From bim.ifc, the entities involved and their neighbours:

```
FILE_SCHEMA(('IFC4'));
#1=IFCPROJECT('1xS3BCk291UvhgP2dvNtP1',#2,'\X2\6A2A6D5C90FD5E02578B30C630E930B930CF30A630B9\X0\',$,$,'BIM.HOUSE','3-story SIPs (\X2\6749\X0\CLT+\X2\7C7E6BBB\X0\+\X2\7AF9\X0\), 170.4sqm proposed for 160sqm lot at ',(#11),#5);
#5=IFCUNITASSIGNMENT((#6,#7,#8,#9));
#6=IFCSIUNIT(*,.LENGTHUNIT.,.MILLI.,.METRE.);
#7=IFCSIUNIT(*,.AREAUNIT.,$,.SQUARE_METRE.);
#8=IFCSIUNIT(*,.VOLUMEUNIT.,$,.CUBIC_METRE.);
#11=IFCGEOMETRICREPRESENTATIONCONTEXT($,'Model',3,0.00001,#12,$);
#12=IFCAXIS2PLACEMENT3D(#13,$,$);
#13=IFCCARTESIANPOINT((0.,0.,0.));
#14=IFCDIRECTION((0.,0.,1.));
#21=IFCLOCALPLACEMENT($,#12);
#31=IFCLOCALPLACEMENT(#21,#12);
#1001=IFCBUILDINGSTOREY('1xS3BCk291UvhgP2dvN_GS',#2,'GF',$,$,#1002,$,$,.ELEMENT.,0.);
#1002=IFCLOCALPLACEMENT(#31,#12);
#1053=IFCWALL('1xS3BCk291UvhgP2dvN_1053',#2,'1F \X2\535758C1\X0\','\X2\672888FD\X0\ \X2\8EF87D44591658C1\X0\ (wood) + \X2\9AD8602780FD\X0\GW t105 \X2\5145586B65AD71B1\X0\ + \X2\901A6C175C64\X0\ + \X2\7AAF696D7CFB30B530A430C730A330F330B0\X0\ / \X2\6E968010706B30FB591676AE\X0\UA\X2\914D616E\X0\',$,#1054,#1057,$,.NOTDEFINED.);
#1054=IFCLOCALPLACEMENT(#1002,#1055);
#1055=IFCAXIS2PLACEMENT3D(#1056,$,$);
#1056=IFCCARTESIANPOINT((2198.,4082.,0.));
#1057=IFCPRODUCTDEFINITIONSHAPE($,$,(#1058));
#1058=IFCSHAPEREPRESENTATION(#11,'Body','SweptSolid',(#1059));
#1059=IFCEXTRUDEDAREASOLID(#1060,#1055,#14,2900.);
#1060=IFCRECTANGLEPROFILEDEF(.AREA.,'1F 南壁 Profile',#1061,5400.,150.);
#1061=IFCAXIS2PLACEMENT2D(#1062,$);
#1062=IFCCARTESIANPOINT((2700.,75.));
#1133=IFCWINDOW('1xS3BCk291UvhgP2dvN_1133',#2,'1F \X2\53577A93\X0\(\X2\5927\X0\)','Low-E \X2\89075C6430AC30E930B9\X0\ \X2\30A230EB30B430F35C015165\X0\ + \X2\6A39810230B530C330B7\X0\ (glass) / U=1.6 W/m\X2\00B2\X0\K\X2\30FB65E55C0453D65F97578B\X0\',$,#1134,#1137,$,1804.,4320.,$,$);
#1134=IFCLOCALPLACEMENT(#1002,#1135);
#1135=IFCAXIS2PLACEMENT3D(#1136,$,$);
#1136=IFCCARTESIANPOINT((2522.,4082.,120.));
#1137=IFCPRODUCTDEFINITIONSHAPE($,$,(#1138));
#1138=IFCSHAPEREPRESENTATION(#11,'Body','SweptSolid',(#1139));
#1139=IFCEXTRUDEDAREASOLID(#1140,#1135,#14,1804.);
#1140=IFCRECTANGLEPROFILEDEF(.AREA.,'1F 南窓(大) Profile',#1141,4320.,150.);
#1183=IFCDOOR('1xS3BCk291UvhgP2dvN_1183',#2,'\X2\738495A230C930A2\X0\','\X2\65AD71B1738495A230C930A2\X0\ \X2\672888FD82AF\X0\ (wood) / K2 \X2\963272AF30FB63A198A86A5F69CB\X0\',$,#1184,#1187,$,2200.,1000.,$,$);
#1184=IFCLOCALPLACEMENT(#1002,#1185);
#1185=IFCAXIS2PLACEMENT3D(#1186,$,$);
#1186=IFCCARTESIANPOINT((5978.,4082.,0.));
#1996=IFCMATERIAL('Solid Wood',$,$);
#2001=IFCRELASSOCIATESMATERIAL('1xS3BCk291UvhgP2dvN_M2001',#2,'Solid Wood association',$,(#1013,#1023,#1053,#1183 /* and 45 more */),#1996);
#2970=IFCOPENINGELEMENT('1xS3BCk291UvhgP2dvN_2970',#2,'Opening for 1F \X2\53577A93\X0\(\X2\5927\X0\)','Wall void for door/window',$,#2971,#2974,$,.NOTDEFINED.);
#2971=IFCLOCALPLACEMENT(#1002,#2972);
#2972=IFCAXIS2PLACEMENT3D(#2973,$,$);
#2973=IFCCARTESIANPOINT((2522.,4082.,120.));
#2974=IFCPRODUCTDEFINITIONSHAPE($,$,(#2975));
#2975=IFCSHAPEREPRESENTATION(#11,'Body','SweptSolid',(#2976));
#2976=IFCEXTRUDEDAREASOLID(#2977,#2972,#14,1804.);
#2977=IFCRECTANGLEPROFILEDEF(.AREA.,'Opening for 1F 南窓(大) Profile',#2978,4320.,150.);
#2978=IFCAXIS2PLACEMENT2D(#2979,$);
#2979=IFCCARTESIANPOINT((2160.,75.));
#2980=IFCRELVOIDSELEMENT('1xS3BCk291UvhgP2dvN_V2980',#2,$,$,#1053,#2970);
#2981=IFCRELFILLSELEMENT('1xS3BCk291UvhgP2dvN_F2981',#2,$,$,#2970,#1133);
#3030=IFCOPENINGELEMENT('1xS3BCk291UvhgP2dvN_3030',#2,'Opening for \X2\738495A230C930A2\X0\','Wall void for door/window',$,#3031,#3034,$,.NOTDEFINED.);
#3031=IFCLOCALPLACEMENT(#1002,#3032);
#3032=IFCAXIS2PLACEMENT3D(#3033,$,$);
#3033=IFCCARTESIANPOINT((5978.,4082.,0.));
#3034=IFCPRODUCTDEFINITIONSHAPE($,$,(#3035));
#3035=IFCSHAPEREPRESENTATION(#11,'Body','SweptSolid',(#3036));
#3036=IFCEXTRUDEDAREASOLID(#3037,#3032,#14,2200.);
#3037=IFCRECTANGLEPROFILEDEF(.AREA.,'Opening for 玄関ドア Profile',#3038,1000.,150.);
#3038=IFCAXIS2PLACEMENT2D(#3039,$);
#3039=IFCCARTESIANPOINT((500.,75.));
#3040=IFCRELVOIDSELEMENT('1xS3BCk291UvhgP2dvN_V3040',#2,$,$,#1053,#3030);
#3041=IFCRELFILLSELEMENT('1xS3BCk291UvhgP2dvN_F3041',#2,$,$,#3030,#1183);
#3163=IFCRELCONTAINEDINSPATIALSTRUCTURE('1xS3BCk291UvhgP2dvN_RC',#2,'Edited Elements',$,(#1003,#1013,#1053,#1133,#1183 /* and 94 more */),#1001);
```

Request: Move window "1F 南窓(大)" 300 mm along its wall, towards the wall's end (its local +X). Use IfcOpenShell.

```python
import ifcopenshell
import ifcopenshell.api.geometry
import ifcopenshell.util.placement
import ifcopenshell.util.unit

model = ifcopenshell.open("bim.ifc")
unit_scale = ifcopenshell.util.unit.calculate_unit_scale(model)

window = model.by_guid("1xS3BCk291UvhgP2dvN_1133")
opening = window.FillsVoids[0].RelatingOpeningElement
wall = opening.VoidsElements[0].RelatingBuildingElement

wall_matrix = ifcopenshell.util.placement.get_local_placement(wall.ObjectPlacement)
shift = wall_matrix[:3, 0] * 0.3 / unit_scale
before = ifcopenshell.util.placement.get_local_placement(window.ObjectPlacement)[:3, 3].copy()

# The window is not placed relative to its opening, so move both.
for product in (opening, window):
    matrix = ifcopenshell.util.placement.get_local_placement(product.ObjectPlacement)
    matrix[:3, 3] += shift
    ifcopenshell.api.geometry.edit_object_placement(model, product=product, matrix=matrix, is_si=False)

after = ifcopenshell.util.placement.get_local_placement(window.ObjectPlacement)[:3, 3]
print("window moved by", (after - before).round(3) + 0.0)

model.write("bim-out.ifc")
```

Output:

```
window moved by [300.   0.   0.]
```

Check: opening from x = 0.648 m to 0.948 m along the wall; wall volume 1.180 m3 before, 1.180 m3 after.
